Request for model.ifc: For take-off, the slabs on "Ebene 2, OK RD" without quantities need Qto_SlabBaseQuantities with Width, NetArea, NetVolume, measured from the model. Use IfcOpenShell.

First a look at what the model holds.

```python
import ifcopenshell
import ifcopenshell.util.element
import ifcopenshell.util.unit

model = ifcopenshell.open("model.ifc")
print(model.schema)
for unit_type in ("LENGTHUNIT", "AREAUNIT", "VOLUMEUNIT"):
    print(unit_type, ifcopenshell.util.unit.calculate_unit_scale(model, unit_type))
storey = next(s for s in model.by_type("IfcBuildingStorey") if s.Name == "Ebene 2, OK RD")
slabs = [e for e in ifcopenshell.util.element.get_decomposition(storey) if e.is_a("IfcSlab")]
for e in sorted(slabs, key=lambda e: e.id()):
    print(e.id(), e.is_a(), e.Name, list(ifcopenshell.util.element.get_psets(e, qtos_only=True)), sep=" | ")
```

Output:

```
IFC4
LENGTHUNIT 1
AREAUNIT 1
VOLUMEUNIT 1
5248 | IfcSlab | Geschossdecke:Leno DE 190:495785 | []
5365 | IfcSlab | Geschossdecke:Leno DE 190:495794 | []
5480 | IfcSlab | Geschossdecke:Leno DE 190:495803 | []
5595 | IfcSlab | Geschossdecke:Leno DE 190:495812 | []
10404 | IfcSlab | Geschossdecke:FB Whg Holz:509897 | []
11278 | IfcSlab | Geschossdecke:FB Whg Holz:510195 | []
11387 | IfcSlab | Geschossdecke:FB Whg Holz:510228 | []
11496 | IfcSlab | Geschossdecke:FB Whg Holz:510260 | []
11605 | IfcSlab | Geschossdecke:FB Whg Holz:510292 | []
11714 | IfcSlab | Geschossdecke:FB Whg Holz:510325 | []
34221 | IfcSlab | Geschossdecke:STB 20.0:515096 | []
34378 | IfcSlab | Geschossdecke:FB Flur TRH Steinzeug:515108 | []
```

```python
import ifcopenshell
import ifcopenshell.api.pset
import ifcopenshell.geom
import ifcopenshell.util.element
import ifcopenshell.util.shape
import ifcopenshell.util.unit

model = ifcopenshell.open("model.ifc")
unit_scale = ifcopenshell.util.unit.calculate_unit_scale(model)
area_scale = ifcopenshell.util.unit.calculate_unit_scale(model, "AREAUNIT")
volume_scale = ifcopenshell.util.unit.calculate_unit_scale(model, "VOLUMEUNIT")
settings = ifcopenshell.geom.settings()

storey = next(s for s in model.by_type("IfcBuildingStorey") if s.Name == "Ebene 2, OK RD")
slabs = [e for e in ifcopenshell.util.element.get_decomposition(storey) if e.is_a("IfcSlab")]

for e in sorted(slabs, key=lambda e: e.id()):
    if ifcopenshell.util.element.get_psets(e, qtos_only=True, should_inherit=False):
        continue
    # Geometry comes back in metres, in the element's own axes.
    shape = ifcopenshell.geom.create_shape(settings, e)
    values = {
        "Width": ifcopenshell.util.shape.get_z(shape.geometry) / unit_scale,
        "NetArea": ifcopenshell.util.shape.get_footprint_area(shape.geometry) / area_scale,
        "NetVolume": ifcopenshell.util.shape.get_volume(shape.geometry) / volume_scale,
    }
    qto = ifcopenshell.api.pset.add_qto(model, product=e, name="Qto_SlabBaseQuantities")
    ifcopenshell.api.pset.edit_qto(model, qto=qto, properties=values)
    print(e.id(), {k: round(v, 3) for k, v in values.items()})

model.write("model_edited.ifc")
```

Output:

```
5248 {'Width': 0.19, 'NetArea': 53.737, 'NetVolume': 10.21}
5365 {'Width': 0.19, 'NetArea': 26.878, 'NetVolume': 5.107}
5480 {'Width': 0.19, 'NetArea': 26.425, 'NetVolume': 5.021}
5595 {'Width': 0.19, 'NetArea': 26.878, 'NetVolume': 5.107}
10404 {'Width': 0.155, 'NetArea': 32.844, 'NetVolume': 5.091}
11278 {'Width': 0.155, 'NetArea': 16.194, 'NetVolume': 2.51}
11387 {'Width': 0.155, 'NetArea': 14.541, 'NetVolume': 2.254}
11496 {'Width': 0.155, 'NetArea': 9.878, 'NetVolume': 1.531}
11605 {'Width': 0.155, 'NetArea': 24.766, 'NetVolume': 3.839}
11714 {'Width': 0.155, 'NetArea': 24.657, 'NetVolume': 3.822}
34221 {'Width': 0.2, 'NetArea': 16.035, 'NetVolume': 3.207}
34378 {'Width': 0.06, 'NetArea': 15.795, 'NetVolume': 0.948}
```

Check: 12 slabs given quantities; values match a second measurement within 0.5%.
